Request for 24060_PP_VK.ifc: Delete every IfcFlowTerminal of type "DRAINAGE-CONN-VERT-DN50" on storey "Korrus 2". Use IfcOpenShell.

First a look at what the model holds.

```python
import ifcopenshell
import ifcopenshell.util.element

model = ifcopenshell.open("24060_PP_VK.ifc")
print(model.schema)
storey = next(s for s in model.by_type("IfcBuildingStorey") if s.Name == "Korrus 2")
terminals = [e for e in ifcopenshell.util.element.get_decomposition(storey) if e.is_a("IfcFlowTerminal")]
seen = {}
for e in terminals:
    element_type = ifcopenshell.util.element.get_type(e)
    name = element_type.Name if element_type not in (None, e) else None
    seen[name] = seen.get(name, 0) + 1
for name, count in sorted(seen.items(), key=str):
    print(count, "x", name)
```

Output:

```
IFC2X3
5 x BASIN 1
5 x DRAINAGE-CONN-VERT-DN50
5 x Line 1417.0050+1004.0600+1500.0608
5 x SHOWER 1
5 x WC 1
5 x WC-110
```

```python
import ifcopenshell
import ifcopenshell.api.root
import ifcopenshell.util.element

model = ifcopenshell.open("24060_PP_VK.ifc")

storey = next(s for s in model.by_type("IfcBuildingStorey") if s.Name == "Korrus 2")
terminals = [e for e in ifcopenshell.util.element.get_decomposition(storey) if e.is_a("IfcFlowTerminal")]
targets = [e for e in terminals if (t := ifcopenshell.util.element.get_type(e)) not in (None, e) and t.Name == "DRAINAGE-CONN-VERT-DN50"]

for e in targets:
    ifcopenshell.api.root.remove_product(model, product=e)
print(len(targets), "removed")

model.write("24060_PP_VK_updated.ifc")
```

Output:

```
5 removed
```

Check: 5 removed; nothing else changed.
